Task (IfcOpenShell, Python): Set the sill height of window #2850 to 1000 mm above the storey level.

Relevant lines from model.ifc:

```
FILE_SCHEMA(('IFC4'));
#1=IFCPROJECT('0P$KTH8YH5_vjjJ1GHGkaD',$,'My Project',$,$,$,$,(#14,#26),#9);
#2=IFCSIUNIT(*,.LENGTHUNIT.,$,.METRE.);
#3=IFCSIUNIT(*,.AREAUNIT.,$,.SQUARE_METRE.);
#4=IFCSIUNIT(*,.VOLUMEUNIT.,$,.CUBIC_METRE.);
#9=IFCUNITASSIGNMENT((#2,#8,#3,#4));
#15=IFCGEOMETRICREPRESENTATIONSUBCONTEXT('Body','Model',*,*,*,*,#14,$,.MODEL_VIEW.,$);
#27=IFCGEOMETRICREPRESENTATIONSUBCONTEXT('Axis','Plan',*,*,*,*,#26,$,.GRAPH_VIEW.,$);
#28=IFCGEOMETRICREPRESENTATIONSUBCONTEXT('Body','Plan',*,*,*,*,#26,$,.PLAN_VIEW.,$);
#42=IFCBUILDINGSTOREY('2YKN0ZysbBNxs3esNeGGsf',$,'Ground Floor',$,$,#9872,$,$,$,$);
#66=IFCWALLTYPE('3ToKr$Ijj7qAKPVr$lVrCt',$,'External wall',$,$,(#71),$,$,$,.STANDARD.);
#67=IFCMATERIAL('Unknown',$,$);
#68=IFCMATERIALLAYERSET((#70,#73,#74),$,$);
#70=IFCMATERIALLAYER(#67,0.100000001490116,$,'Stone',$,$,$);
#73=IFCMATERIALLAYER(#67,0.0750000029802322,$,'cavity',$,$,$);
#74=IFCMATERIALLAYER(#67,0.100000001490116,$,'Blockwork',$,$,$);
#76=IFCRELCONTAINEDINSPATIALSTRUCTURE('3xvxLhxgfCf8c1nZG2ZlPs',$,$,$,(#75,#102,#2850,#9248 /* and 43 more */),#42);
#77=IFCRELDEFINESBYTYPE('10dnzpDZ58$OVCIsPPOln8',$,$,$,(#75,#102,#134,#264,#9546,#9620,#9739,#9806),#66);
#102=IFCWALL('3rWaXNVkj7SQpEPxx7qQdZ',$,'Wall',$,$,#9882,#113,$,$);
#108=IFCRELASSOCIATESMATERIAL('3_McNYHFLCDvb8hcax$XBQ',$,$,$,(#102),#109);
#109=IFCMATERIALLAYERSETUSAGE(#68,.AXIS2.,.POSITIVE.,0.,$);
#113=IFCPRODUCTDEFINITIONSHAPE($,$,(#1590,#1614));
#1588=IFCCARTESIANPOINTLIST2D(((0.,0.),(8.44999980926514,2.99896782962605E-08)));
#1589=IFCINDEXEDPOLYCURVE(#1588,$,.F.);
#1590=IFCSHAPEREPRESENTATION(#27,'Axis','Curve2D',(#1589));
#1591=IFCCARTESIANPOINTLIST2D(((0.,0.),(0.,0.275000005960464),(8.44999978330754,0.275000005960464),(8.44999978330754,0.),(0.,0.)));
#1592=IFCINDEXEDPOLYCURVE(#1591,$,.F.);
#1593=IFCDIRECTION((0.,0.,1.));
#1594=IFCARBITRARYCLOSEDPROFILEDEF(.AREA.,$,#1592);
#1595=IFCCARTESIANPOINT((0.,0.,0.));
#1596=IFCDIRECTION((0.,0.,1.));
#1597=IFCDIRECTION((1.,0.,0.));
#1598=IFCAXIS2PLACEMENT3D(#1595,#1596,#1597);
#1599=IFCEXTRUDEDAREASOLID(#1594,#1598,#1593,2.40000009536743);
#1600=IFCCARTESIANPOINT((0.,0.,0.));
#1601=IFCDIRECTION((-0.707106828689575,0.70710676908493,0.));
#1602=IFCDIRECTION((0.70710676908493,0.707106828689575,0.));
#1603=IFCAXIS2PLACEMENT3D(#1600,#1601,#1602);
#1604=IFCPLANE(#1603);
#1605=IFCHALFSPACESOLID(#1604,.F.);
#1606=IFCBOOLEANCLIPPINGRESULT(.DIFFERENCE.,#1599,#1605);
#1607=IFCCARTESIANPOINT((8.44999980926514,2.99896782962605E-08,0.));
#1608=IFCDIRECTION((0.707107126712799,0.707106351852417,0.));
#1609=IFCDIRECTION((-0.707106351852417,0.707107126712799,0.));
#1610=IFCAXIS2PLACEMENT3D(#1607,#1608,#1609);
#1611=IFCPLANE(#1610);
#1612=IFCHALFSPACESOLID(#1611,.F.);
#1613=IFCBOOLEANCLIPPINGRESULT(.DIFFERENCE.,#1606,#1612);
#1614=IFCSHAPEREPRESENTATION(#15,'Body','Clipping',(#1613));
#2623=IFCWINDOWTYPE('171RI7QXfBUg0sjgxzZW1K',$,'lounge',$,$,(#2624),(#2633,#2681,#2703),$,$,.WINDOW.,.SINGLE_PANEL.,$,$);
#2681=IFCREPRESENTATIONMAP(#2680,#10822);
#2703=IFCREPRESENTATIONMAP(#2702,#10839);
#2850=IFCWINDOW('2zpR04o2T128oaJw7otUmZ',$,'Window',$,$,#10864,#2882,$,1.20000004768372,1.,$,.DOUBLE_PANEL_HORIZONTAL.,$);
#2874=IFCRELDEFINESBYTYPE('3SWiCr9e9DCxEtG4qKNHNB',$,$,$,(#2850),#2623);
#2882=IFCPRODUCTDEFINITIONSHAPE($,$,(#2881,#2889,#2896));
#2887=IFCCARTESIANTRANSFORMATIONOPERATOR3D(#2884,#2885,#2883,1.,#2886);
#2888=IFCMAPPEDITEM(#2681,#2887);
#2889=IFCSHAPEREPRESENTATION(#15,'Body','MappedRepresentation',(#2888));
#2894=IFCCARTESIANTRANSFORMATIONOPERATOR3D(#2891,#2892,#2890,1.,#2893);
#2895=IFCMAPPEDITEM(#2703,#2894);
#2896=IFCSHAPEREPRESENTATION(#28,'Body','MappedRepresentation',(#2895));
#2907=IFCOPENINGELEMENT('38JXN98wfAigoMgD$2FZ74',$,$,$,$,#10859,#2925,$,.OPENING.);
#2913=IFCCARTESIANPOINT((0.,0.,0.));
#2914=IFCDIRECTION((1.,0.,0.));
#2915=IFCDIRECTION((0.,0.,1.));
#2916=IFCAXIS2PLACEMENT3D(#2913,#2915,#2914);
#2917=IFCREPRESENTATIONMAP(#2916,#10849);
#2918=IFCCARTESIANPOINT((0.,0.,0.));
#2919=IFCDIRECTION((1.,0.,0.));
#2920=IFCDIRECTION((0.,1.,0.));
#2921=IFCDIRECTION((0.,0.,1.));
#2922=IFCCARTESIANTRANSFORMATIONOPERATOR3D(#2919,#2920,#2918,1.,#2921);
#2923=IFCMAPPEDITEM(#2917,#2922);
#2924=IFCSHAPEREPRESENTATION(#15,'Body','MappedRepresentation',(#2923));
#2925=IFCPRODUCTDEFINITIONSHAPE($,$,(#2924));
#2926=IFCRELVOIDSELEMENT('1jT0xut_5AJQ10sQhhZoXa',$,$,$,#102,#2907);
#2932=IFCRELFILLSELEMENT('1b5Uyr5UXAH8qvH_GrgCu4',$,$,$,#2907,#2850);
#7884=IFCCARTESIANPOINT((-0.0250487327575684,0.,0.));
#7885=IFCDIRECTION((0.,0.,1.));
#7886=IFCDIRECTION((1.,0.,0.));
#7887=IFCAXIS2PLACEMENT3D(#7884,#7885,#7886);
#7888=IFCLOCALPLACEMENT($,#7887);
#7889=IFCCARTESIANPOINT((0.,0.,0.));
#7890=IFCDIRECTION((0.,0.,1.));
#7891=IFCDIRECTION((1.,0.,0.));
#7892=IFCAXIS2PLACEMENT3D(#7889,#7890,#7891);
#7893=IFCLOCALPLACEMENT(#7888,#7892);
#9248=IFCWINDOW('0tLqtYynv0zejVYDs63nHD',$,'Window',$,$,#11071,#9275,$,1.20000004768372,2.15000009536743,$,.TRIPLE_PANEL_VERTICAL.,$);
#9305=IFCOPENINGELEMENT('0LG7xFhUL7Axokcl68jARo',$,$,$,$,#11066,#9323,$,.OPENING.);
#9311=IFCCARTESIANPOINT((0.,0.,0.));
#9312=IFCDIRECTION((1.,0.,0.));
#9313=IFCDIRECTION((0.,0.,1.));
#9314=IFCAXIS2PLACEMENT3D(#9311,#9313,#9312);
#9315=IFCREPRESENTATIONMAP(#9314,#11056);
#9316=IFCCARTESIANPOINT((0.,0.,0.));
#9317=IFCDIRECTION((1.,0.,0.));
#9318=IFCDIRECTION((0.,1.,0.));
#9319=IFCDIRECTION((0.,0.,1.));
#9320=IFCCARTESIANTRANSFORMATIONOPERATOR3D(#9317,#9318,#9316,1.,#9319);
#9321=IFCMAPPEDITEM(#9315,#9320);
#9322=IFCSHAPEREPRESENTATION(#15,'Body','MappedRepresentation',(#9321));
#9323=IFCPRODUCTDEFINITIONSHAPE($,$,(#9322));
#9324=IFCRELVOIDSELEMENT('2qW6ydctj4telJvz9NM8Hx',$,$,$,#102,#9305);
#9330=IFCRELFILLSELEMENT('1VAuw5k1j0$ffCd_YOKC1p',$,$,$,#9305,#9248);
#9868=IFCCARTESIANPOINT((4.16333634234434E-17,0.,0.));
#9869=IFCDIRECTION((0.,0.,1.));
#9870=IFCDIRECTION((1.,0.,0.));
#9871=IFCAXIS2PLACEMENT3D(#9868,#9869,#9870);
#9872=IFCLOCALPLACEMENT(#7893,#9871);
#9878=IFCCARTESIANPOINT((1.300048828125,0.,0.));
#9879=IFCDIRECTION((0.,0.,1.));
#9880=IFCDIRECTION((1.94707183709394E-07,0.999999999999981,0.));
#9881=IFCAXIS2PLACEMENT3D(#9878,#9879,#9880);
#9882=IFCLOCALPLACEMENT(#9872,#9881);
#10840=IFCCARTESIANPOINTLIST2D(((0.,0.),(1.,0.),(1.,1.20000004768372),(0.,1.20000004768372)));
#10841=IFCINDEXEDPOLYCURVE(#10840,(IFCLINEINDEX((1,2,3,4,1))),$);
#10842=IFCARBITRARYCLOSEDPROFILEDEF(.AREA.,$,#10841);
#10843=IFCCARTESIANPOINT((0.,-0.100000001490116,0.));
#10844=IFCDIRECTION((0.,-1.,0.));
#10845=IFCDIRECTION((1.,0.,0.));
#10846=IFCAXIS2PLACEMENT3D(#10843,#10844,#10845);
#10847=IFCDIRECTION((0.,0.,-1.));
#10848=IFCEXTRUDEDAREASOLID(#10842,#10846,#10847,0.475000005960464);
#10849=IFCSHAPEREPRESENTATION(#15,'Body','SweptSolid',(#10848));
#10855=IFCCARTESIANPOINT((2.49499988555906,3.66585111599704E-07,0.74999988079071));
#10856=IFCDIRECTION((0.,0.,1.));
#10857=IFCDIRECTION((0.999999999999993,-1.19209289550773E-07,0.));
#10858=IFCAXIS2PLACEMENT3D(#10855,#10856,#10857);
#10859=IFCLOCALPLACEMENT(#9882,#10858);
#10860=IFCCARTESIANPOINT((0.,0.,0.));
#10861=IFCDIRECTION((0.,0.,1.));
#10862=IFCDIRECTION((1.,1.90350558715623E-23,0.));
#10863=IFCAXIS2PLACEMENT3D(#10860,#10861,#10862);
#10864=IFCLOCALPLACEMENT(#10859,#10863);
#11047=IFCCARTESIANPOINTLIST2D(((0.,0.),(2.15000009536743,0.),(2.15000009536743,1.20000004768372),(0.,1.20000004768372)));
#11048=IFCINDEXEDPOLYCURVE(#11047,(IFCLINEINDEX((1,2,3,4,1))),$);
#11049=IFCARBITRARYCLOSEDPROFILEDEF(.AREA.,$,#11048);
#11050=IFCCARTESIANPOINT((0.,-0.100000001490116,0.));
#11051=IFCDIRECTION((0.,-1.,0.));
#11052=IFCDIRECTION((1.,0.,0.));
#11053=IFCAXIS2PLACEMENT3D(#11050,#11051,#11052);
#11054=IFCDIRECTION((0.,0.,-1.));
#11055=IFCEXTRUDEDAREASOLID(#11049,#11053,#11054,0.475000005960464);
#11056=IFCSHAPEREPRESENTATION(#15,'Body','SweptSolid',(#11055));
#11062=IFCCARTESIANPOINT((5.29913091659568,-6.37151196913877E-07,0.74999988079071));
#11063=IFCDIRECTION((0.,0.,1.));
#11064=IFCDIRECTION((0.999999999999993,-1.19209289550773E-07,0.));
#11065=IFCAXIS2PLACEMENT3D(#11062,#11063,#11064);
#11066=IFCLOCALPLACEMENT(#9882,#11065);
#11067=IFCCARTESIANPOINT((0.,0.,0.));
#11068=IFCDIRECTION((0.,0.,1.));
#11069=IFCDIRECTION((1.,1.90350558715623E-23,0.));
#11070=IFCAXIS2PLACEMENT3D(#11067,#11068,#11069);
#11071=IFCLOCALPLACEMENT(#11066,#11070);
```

```python
import numpy as np
import ifcopenshell
import ifcopenshell.api.geometry
import ifcopenshell.geom
import ifcopenshell.util.element
import ifcopenshell.util.placement
import ifcopenshell.util.shape
import ifcopenshell.util.unit

model = ifcopenshell.open("model.ifc")
unit_scale = ifcopenshell.util.unit.calculate_unit_scale(model)

window = model.by_guid("2zpR04o2T128oaJw7otUmZ")
opening = window.FillsVoids[0].RelatingOpeningElement
storey = ifcopenshell.util.element.get_container(window, ifc_class="IfcBuildingStorey")
level = ifcopenshell.util.placement.get_local_placement(storey.ObjectPlacement)[2, 3]

# The opening's origin need not be at the sill, so measure its lowest point.
shape = ifcopenshell.geom.create_shape(ifcopenshell.geom.settings(), opening)
bottom = ifcopenshell.util.shape.get_shape_bottom_elevation(shape, shape.geometry) / unit_scale
dz = level + 1 / unit_scale - bottom

shift = np.array([0.0, 0.0, dz])
# The window is placed relative to its opening, so it follows when the opening moves.
matrix = ifcopenshell.util.placement.get_local_placement(opening.ObjectPlacement)
matrix[:3, 3] += shift
ifcopenshell.api.geometry.edit_object_placement(
    model, product=opening, matrix=matrix, is_si=False, should_transform_children=True
)

print(f"moved by {dz * unit_scale:+.3f} m")

model.write("model_edited.ifc")
```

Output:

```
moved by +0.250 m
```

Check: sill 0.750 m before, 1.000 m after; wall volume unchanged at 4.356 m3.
